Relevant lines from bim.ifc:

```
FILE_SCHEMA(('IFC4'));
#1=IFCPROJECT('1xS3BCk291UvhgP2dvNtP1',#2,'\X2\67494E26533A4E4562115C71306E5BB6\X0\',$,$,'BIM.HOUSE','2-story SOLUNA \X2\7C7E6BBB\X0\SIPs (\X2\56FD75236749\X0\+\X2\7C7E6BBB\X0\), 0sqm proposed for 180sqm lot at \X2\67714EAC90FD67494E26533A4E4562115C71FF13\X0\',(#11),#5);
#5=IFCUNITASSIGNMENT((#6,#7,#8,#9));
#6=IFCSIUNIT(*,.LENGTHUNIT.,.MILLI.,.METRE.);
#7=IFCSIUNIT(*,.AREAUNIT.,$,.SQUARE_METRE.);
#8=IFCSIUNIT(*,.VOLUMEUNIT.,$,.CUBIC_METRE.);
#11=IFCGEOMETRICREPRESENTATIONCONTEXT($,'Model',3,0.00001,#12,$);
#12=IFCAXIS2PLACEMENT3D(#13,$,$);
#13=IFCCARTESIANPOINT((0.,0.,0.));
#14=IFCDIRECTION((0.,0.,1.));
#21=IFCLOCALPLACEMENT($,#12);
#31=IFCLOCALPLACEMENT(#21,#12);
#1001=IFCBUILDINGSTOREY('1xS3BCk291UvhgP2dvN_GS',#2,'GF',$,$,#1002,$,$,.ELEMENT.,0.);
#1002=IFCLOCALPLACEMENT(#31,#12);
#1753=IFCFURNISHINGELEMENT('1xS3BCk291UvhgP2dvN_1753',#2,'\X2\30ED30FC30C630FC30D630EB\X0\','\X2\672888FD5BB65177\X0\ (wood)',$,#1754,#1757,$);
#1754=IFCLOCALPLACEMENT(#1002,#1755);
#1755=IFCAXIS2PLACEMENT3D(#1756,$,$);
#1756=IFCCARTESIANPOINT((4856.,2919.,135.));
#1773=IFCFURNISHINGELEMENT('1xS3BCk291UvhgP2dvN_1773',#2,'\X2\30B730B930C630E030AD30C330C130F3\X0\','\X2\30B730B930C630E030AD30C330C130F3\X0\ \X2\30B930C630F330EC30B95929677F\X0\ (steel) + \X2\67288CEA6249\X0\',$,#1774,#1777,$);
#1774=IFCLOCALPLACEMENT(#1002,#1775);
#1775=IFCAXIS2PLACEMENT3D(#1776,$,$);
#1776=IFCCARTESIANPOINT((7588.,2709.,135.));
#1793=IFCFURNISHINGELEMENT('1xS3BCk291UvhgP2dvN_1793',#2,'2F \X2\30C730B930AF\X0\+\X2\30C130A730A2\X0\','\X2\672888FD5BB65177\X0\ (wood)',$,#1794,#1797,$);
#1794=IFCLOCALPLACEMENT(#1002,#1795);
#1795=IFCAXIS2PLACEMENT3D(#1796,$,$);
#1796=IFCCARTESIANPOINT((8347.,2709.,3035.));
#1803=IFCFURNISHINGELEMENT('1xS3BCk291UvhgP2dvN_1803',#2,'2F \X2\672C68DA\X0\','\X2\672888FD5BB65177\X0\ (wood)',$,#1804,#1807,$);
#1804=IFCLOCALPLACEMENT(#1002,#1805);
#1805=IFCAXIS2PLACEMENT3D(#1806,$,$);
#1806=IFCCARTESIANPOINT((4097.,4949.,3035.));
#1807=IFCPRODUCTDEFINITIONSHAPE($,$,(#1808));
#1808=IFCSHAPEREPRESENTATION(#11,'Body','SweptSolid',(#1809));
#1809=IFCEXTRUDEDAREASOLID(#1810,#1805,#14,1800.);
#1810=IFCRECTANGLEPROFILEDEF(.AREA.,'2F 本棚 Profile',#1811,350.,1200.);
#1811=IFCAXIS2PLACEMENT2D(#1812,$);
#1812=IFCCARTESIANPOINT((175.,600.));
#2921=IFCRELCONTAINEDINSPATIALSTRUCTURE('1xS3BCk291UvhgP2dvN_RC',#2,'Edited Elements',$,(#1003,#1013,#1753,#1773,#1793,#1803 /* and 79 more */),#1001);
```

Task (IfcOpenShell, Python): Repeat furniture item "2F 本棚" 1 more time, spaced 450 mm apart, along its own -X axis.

```python
import ifcopenshell
import ifcopenshell.api.geometry
import ifcopenshell.api.root
import ifcopenshell.util.element
import ifcopenshell.util.placement

model = ifcopenshell.open("bim.ifc")


def reuse_history(source, copy):
    """copy_class also copies each property set's owner history, people and application; keep the originals."""
    for rel in copy.IsDefinedBy:
        if rel.is_a("IfcRelDefinesByProperties") and (history := rel.RelatingPropertyDefinition.OwnerHistory):
            rel.RelatingPropertyDefinition.OwnerHistory = source.OwnerHistory
            ifcopenshell.util.element.remove_deep2(model, history)


source = model.by_guid("1xS3BCk291UvhgP2dvN_1803")
base = ifcopenshell.util.placement.get_local_placement(source.ObjectPlacement)
step = -base[:3, 0] * 450.0

for i in range(1, 2):
    copy = ifcopenshell.api.root.copy_class(model, product=source)
    copy.Representation = ifcopenshell.util.element.copy_deep(
        model, source.Representation, exclude=["IfcGeometricRepresentationContext", "IfcRepresentationMap"]
    )
    reuse_history(source, copy)
    matrix = base.copy()
    matrix[:3, 3] += i * step
    print("added at", matrix[:3, 3].round(3) + 0.0)
    ifcopenshell.api.geometry.edit_object_placement(model, product=copy, matrix=matrix, is_si=False)

model.write("bim_v2.ifc")
```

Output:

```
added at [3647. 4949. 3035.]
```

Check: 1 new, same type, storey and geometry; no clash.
